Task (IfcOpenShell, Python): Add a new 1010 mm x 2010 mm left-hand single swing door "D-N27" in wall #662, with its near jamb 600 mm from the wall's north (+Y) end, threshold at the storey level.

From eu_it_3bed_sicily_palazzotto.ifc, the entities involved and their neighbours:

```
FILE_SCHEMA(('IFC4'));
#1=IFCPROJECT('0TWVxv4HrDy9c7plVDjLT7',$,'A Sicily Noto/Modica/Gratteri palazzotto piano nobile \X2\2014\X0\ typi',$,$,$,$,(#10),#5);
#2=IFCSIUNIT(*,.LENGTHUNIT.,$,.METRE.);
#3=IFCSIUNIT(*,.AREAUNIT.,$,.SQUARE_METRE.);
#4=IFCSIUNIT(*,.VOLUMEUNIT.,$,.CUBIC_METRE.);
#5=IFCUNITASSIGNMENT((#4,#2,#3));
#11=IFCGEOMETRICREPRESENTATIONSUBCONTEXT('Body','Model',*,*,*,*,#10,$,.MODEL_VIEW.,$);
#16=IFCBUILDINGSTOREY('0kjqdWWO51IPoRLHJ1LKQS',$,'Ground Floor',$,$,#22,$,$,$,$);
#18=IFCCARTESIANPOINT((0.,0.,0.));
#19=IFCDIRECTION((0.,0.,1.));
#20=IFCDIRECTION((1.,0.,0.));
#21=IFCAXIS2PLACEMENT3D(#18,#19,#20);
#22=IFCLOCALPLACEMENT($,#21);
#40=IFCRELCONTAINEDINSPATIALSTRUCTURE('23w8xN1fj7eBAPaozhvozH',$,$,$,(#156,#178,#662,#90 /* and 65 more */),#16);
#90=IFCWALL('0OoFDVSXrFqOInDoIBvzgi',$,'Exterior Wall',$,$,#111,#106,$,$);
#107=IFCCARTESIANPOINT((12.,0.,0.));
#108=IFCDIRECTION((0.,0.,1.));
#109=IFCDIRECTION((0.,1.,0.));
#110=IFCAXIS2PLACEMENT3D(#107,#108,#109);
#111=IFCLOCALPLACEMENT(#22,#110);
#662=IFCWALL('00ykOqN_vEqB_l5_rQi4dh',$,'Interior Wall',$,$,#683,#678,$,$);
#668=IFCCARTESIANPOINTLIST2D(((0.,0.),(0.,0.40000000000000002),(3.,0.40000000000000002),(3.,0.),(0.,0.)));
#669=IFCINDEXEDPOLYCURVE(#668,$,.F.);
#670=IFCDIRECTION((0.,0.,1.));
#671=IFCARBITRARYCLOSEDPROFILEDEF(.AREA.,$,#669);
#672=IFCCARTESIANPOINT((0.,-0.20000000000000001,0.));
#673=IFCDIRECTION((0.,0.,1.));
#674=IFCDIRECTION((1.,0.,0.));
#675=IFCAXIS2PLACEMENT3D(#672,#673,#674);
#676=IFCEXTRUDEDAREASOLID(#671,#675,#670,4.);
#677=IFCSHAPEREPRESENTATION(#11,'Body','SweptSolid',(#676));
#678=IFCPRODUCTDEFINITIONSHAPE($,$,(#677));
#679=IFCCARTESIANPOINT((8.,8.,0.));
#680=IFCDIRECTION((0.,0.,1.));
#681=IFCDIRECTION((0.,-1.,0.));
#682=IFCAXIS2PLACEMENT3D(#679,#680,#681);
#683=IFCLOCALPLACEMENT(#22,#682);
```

```python
import numpy as np
import ifcopenshell
import ifcopenshell.api.feature
import ifcopenshell.api.geometry
import ifcopenshell.api.root
import ifcopenshell.api.spatial
import ifcopenshell.geom
import ifcopenshell.util.element
import ifcopenshell.util.placement
import ifcopenshell.util.representation
import ifcopenshell.util.shape
import ifcopenshell.util.unit

model = ifcopenshell.open("eu_it_3bed_sicily_palazzotto.ifc")
unit_scale = ifcopenshell.util.unit.calculate_unit_scale(model)
settings = ifcopenshell.geom.settings()


def volume(element):
    """Net volume in cubic metres, openings subtracted."""
    shape = ifcopenshell.geom.create_shape(settings, element)
    return ifcopenshell.util.shape.get_volume(shape.geometry)


wall = model.by_id(662)
storey = ifcopenshell.util.element.get_container(wall, ifc_class="IfcBuildingStorey")
context = ifcopenshell.util.representation.get_context(model, "Model", "Body", "MODEL_VIEW")
before = volume(wall)

width, height, from_end, sill = 1.01, 2.01, 0.6, 0.0  # metres

# The wall runs along its own X axis, and the end named is its -X end.
wall_shape = ifcopenshell.geom.create_shape(settings, wall)
x, y, z = ifcopenshell.util.shape.get_vertices(wall_shape.geometry).T
start = x.min() + from_end
face, thickness = float(y.min()), float(y.max() - y.min())
wall_matrix = ifcopenshell.util.placement.get_local_placement(wall.ObjectPlacement)
level = ifcopenshell.util.placement.get_local_placement(storey.ObjectPlacement)[2, 3]


def in_wall(x, y):
    """Placement at x, y metres in the wall's axes, at sill height."""
    matrix = wall_matrix.copy()
    matrix[:, 3] = wall_matrix @ np.array([x / unit_scale, y / unit_scale, 0.0, 1.0])
    matrix[2, 3] = level + sill / unit_scale
    return matrix


# Opening: a box that overshoots both wall faces by 50 mm.
opening = ifcopenshell.api.root.create_entity(model, ifc_class="IfcOpeningElement", predefined_type="OPENING")
box = ifcopenshell.api.geometry.add_wall_representation(
    model, context=context, length=width, height=height, thickness=thickness + 0.1
)
ifcopenshell.api.geometry.assign_representation(model, product=opening, representation=box)
ifcopenshell.api.geometry.edit_object_placement(model, product=opening, matrix=in_wall(start, face - 0.05), is_si=False)
ifcopenshell.api.feature.add_feature(model, feature=opening, element=wall)

door = ifcopenshell.api.root.create_entity(model, ifc_class="IfcDoor", name="D-N27", predefined_type="DOOR")
door.OverallWidth, door.OverallHeight = width / unit_scale, height / unit_scale
door.OperationType = "SINGLE_SWING_LEFT"
body = ifcopenshell.api.geometry.add_door_representation(
    model,
    context=context,
    overall_width=door.OverallWidth,
    overall_height=door.OverallHeight,
    operation_type="SINGLE_SWING_LEFT",
    lining_properties={"LiningDepth": thickness / unit_scale, "ThresholdDepth": thickness / unit_scale},
)
ifcopenshell.api.geometry.assign_representation(model, product=door, representation=body)
ifcopenshell.api.spatial.assign_container(model, products=[door], relating_structure=storey)
ifcopenshell.api.feature.add_filling(model, opening=opening, element=door)

# The lining spans the wall, so the door starts at the wall face.
ifcopenshell.api.geometry.edit_object_placement(model, product=door, matrix=in_wall(start, face), is_si=False)

after = volume(wall)

print(f"wall volume {before:.3f} -> {after:.3f} m3")

model.write("eu_it_3bed_sicily_palazzotto_updated.ifc")
```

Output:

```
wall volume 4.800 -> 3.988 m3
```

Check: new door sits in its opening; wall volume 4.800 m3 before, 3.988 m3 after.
